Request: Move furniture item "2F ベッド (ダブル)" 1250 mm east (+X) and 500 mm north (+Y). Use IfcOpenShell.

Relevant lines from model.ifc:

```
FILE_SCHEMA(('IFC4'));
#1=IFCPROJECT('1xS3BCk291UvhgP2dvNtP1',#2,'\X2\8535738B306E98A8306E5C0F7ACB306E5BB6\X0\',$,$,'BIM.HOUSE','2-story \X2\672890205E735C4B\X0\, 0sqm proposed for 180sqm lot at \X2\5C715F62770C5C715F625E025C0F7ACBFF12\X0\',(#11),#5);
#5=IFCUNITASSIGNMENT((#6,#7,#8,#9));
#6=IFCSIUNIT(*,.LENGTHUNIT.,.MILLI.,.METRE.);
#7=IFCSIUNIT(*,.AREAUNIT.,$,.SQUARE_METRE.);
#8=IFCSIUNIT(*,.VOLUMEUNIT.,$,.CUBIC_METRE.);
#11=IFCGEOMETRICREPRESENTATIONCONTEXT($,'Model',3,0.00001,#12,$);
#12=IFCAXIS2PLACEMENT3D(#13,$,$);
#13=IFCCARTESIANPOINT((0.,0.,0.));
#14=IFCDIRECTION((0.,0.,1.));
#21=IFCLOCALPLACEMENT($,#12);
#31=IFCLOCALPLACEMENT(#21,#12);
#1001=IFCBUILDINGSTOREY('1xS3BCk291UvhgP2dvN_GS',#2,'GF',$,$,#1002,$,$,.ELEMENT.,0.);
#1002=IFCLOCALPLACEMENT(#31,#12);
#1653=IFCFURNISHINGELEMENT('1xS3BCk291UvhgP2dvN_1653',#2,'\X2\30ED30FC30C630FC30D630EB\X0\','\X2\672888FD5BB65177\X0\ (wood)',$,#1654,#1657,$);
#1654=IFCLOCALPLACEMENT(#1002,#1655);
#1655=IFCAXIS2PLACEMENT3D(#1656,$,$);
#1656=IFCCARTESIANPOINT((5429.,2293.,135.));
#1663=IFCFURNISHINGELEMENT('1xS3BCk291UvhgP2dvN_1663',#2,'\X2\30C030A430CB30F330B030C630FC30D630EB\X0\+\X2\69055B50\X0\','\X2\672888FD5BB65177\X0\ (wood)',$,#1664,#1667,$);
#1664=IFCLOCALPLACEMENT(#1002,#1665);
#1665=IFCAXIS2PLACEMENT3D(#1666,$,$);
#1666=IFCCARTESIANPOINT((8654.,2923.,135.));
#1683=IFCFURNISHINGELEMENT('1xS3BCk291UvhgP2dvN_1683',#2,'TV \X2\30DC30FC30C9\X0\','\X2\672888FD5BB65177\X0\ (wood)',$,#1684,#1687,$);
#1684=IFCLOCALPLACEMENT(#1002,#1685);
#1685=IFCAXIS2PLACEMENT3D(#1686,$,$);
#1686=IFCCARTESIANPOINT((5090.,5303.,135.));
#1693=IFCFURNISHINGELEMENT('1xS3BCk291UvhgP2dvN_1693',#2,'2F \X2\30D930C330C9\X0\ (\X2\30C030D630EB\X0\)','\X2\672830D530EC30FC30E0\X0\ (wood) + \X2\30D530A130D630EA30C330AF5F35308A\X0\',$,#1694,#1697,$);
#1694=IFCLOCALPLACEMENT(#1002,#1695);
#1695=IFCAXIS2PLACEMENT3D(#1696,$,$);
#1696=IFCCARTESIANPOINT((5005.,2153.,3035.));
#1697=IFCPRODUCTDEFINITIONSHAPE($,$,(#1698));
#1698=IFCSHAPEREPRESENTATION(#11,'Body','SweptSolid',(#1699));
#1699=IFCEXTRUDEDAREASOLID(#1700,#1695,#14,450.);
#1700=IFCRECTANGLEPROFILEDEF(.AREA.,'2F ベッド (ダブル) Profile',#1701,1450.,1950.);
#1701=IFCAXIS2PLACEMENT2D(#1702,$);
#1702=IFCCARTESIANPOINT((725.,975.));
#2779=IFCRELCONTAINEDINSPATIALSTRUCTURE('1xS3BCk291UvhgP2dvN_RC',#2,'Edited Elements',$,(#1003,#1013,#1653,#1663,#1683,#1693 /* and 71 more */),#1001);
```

```python
import ifcopenshell
import ifcopenshell.api.geometry
import ifcopenshell.util.placement

model = ifcopenshell.open("model.ifc")

item = model.by_guid("1xS3BCk291UvhgP2dvN_1693")
matrix = ifcopenshell.util.placement.get_local_placement(item.ObjectPlacement)
matrix[0, 3] += 1250.0
matrix[1, 3] += 500.0
ifcopenshell.api.geometry.edit_object_placement(model, product=item, matrix=matrix, is_si=False)

print(ifcopenshell.util.placement.get_local_placement(item.ObjectPlacement).round(3) + 0.0)

model.write("model_v2.ifc")
```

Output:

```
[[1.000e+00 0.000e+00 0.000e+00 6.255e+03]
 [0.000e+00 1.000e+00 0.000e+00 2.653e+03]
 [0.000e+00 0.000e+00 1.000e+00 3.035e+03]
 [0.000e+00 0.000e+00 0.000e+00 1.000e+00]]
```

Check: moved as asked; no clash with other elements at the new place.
